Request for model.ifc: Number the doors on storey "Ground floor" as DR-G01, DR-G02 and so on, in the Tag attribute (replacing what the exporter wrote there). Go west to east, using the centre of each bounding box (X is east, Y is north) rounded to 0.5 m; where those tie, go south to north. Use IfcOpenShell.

First a look at what the model holds.

```python
import ifcopenshell
import ifcopenshell.util.element
import ifcopenshell.util.placement

model = ifcopenshell.open("model.ifc")
print(model.schema)
storey = next(s for s in model.by_type("IfcBuildingStorey") if s.Name == "Ground floor")
doors = [e for e in ifcopenshell.util.element.get_decomposition(storey) if e.is_a("IfcDoor")]
for e in sorted(doors, key=lambda e: e.id()):
    origin = ifcopenshell.util.placement.get_local_placement(e.ObjectPlacement)[:3, 3]
    print(e.id(), e.Tag, e.Name, origin.round(2) + 0.0, sep=" | ")
```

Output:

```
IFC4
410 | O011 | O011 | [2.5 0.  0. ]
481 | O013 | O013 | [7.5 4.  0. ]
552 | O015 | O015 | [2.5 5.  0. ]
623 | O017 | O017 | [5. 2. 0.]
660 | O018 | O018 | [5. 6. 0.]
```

```python
import ifcopenshell
import ifcopenshell.geom
import ifcopenshell.util.element
import ifcopenshell.util.shape

model = ifcopenshell.open("model.ifc")
settings = ifcopenshell.geom.settings()
settings.set("use-world-coords", True)


def centre(element):
    shape = ifcopenshell.geom.create_shape(settings, element)
    return ifcopenshell.util.shape.get_bbox_centroid(shape.geometry)


storey = next(s for s in model.by_type("IfcBuildingStorey") if s.Name == "Ground floor")
doors = [e for e in ifcopenshell.util.element.get_decomposition(storey) if e.is_a("IfcDoor")]

# Insertion points can sit at a corner or the storey origin, so sort by the geometry (in metres).
centres = {e: centre(e) for e in doors}
doors.sort(key=lambda e: (round(centres[e][0] / 0.5), centres[e][1]))

for i, e in enumerate(doors, start=1):
    number = f"DR-G{i:02d}"
    e.Tag = number
    print(e.id(), number)

model.write("model_updated.ifc")
```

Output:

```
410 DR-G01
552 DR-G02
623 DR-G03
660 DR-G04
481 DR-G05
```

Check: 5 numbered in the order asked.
